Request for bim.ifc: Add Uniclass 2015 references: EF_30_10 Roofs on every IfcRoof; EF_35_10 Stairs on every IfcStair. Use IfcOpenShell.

First a look at what the model holds.

```python
import ifcopenshell

model = ifcopenshell.open("bim.ifc")
print(model.schema)
print("classifications:", [c.Name for c in model.by_type("IfcClassification")])
for ifc_class in ("IfcDoor", "IfcRoof", "IfcStair", "IfcWall", "IfcWindow"):
    print(ifc_class, len(model.by_type(ifc_class)))
```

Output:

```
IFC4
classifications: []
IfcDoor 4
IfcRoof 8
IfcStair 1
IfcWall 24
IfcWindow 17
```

```python
import ifcopenshell
import ifcopenshell.api.classification

model = ifcopenshell.open("bim.ifc")

system = ifcopenshell.api.classification.add_classification(model, classification="Uniclass 2015")

codes = {
    "IfcRoof": ("EF_30_10", "Roofs"),
    "IfcStair": ("EF_35_10", "Stairs"),
}
for ifc_class, (code, name) in codes.items():
    products = model.by_type(ifc_class)
    ifcopenshell.api.classification.add_reference(
        model, products=products, classification=system, identification=code, name=name
    )
    print(code, len(products))

model.write("bim_edited.ifc")
```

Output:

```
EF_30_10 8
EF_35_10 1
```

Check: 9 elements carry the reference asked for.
